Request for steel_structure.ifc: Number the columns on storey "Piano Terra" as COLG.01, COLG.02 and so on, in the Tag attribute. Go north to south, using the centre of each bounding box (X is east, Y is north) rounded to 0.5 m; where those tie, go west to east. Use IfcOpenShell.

First a look at what the model holds.

```python
import ifcopenshell
import ifcopenshell.util.element
import ifcopenshell.util.placement

model = ifcopenshell.open("steel_structure.ifc")
print(model.schema)
storey = next(s for s in model.by_type("IfcBuildingStorey") if s.Name == "Piano Terra")
columns = [e for e in ifcopenshell.util.element.get_decomposition(storey) if e.is_a("IfcColumn")]
for e in sorted(columns, key=lambda e: e.id()):
    origin = ifcopenshell.util.placement.get_local_placement(e.ObjectPlacement)[:3, 3]
    print(e.id(), e.Tag, e.Name, origin.round(2) + 0.0, sep=" | ")
```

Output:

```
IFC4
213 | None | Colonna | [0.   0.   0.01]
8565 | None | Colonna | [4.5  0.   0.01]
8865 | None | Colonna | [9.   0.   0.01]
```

```python
import ifcopenshell
import ifcopenshell.geom
import ifcopenshell.util.element
import ifcopenshell.util.shape

model = ifcopenshell.open("steel_structure.ifc")
settings = ifcopenshell.geom.settings()
settings.set("use-world-coords", True)


def centre(element):
    shape = ifcopenshell.geom.create_shape(settings, element)
    return ifcopenshell.util.shape.get_bbox_centroid(shape.geometry)


storey = next(s for s in model.by_type("IfcBuildingStorey") if s.Name == "Piano Terra")
columns = [e for e in ifcopenshell.util.element.get_decomposition(storey) if e.is_a("IfcColumn")]

# Insertion points can sit at a corner or the storey origin, so sort by the geometry (in metres).
centres = {e: centre(e) for e in columns}
columns.sort(key=lambda e: (-round(centres[e][1] / 0.5), centres[e][0]))

for i, e in enumerate(columns, start=1):
    number = f"COLG.{i:02d}"
    e.Tag = number
    print(e.id(), number)

model.write("steel_structure_v2.ifc")
```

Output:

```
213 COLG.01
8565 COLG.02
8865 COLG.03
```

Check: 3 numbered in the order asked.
